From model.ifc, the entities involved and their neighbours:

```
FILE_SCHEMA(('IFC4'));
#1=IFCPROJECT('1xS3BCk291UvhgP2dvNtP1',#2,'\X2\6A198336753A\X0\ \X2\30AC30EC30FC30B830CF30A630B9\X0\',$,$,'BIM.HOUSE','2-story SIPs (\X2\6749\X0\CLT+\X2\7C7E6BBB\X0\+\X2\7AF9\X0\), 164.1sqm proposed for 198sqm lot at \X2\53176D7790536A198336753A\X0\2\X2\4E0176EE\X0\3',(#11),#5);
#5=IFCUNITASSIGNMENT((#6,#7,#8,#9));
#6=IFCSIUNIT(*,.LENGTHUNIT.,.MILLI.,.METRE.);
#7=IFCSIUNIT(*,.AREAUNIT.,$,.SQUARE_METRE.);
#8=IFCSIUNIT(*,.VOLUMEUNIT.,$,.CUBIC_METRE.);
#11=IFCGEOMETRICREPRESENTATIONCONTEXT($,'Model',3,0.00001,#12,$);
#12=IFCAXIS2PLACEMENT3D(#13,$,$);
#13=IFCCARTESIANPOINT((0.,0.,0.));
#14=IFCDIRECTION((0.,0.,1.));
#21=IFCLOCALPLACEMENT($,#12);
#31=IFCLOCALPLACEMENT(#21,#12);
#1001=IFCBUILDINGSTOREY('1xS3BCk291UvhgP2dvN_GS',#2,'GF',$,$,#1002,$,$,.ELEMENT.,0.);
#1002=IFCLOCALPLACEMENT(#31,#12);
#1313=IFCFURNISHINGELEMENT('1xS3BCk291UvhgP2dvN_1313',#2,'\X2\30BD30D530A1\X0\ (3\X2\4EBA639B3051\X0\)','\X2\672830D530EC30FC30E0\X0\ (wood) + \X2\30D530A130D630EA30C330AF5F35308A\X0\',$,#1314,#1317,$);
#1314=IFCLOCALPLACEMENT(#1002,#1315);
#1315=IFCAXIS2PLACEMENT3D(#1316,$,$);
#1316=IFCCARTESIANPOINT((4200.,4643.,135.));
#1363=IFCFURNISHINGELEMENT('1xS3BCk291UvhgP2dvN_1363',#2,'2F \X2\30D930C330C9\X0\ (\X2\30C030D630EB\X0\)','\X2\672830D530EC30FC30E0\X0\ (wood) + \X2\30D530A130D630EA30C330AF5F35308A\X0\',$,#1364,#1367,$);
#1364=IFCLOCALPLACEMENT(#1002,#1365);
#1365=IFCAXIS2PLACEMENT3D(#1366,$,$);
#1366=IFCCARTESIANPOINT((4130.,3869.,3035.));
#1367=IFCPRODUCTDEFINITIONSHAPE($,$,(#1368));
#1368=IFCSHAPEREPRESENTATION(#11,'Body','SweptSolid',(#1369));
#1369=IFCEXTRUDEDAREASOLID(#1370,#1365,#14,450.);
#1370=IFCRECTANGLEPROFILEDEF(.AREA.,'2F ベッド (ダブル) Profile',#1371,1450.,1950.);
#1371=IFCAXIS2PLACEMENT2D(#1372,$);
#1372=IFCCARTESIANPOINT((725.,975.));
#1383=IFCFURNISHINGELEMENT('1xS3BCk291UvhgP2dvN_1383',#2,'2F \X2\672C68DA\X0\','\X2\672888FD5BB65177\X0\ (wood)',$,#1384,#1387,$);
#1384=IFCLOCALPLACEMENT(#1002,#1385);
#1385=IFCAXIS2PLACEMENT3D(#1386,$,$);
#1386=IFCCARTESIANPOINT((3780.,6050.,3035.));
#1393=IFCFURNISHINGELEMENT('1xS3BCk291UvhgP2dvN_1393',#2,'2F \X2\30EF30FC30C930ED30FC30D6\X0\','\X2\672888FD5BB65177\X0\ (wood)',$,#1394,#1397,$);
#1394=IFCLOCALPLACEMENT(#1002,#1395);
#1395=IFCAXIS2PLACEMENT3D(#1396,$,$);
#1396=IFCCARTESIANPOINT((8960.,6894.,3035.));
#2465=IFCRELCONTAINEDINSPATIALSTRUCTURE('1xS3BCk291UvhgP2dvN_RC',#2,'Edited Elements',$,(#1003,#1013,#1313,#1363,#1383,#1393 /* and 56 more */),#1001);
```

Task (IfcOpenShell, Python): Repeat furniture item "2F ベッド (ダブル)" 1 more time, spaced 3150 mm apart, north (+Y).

```python
import numpy as np
import ifcopenshell
import ifcopenshell.api.geometry
import ifcopenshell.api.root
import ifcopenshell.util.element
import ifcopenshell.util.placement
import ifcopenshell.util.unit

model = ifcopenshell.open("model.ifc")
unit_scale = ifcopenshell.util.unit.calculate_unit_scale(model)


def reuse_history(source, copy):
    """copy_class also copies each property set's owner history, people and application; keep the originals."""
    for rel in copy.IsDefinedBy:
        if rel.is_a("IfcRelDefinesByProperties") and (history := rel.RelatingPropertyDefinition.OwnerHistory):
            rel.RelatingPropertyDefinition.OwnerHistory = source.OwnerHistory
            ifcopenshell.util.element.remove_deep2(model, history)


source = model.by_guid("1xS3BCk291UvhgP2dvN_1363")
base = ifcopenshell.util.placement.get_local_placement(source.ObjectPlacement)
step = np.array([0.0, 1.0, 0.0]) * 3.15 / unit_scale

for i in range(1, 2):
    copy = ifcopenshell.api.root.copy_class(model, product=source)
    copy.Representation = ifcopenshell.util.element.copy_deep(
        model, source.Representation, exclude=["IfcGeometricRepresentationContext", "IfcRepresentationMap"]
    )
    reuse_history(source, copy)
    matrix = base.copy()
    matrix[:3, 3] += i * step
    print("added at", matrix[:3, 3].round(3) + 0.0)
    ifcopenshell.api.geometry.edit_object_placement(model, product=copy, matrix=matrix, is_si=False)

model.write("model_edited.ifc")
```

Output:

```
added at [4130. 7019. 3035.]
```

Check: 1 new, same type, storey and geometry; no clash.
